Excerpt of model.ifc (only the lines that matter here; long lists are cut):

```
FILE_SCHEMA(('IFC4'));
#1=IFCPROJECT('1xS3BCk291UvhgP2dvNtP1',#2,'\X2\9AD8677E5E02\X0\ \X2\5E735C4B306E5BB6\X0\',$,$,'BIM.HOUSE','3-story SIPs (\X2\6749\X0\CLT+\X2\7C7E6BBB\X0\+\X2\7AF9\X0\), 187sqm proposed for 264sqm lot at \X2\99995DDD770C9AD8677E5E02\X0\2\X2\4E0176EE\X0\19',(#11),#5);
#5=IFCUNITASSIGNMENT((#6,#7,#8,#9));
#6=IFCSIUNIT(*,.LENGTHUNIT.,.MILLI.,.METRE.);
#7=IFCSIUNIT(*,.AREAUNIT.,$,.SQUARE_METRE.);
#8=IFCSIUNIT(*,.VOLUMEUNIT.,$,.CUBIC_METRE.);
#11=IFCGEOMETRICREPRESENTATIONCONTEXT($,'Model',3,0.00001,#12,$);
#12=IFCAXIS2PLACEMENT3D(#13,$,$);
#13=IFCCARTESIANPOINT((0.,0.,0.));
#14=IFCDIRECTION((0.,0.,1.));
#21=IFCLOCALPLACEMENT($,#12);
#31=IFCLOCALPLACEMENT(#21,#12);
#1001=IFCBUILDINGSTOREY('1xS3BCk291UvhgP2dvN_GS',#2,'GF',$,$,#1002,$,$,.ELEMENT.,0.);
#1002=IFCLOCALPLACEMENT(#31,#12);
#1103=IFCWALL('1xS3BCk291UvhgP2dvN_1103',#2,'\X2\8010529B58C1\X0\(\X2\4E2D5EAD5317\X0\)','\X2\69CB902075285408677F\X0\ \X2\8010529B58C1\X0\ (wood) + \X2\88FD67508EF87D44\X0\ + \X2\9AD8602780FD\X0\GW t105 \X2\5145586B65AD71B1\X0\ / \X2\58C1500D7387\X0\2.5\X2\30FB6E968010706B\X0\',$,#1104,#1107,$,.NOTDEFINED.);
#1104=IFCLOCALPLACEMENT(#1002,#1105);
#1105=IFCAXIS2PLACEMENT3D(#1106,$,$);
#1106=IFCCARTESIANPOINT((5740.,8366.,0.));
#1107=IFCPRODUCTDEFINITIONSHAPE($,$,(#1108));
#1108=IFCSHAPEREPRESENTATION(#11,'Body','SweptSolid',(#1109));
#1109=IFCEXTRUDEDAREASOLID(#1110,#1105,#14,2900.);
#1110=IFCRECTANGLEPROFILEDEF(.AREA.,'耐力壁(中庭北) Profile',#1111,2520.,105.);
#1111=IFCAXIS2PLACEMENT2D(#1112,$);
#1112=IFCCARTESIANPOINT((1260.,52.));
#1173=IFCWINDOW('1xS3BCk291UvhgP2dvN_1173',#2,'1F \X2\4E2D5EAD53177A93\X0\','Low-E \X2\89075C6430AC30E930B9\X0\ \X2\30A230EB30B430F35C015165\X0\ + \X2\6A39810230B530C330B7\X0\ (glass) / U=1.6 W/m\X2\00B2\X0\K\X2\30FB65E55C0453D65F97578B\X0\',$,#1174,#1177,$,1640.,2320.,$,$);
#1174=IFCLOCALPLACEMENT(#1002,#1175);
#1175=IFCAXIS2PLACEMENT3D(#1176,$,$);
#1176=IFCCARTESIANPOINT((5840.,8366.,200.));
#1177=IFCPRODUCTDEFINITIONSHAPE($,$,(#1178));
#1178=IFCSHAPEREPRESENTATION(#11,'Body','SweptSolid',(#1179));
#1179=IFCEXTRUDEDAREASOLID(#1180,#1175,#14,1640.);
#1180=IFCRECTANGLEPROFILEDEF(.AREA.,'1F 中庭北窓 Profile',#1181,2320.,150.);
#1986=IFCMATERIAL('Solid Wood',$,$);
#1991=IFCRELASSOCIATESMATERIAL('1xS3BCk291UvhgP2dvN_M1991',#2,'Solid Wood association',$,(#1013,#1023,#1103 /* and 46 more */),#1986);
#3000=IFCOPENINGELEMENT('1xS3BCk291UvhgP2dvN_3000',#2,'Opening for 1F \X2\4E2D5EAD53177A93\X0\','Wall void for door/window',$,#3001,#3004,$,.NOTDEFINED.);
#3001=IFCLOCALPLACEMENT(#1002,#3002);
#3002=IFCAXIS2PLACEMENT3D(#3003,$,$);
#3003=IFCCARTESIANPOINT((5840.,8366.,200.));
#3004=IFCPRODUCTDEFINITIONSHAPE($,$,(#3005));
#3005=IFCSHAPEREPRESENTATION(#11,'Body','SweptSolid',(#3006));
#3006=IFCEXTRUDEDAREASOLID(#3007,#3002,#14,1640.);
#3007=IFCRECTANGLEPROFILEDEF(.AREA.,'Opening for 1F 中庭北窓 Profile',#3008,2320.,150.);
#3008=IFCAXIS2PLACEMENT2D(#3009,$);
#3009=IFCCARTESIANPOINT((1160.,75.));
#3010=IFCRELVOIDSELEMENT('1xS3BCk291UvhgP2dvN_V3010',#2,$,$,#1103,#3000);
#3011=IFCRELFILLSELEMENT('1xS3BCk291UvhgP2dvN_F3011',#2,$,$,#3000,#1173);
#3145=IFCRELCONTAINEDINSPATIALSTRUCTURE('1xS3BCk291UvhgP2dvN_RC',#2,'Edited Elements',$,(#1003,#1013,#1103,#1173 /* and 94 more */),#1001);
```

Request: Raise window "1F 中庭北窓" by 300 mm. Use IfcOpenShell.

```python
import numpy as np
import ifcopenshell
import ifcopenshell.api.geometry
import ifcopenshell.util.placement
import ifcopenshell.util.unit

model = ifcopenshell.open("model.ifc")
unit_scale = ifcopenshell.util.unit.calculate_unit_scale(model)

window = model.by_guid("1xS3BCk291UvhgP2dvN_1173")
opening = window.FillsVoids[0].RelatingOpeningElement
dz = 0.3 / unit_scale

shift = np.array([0.0, 0.0, dz])
# The window is not placed relative to its opening, so move both.
for product in (opening, window):
    matrix = ifcopenshell.util.placement.get_local_placement(product.ObjectPlacement)
    matrix[:3, 3] += shift
    ifcopenshell.api.geometry.edit_object_placement(model, product=product, matrix=matrix, is_si=False)

print(f"moved by {dz * unit_scale:+.3f} m")

model.write("model_edited.ifc")
```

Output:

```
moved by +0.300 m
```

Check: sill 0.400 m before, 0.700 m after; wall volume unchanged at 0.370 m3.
